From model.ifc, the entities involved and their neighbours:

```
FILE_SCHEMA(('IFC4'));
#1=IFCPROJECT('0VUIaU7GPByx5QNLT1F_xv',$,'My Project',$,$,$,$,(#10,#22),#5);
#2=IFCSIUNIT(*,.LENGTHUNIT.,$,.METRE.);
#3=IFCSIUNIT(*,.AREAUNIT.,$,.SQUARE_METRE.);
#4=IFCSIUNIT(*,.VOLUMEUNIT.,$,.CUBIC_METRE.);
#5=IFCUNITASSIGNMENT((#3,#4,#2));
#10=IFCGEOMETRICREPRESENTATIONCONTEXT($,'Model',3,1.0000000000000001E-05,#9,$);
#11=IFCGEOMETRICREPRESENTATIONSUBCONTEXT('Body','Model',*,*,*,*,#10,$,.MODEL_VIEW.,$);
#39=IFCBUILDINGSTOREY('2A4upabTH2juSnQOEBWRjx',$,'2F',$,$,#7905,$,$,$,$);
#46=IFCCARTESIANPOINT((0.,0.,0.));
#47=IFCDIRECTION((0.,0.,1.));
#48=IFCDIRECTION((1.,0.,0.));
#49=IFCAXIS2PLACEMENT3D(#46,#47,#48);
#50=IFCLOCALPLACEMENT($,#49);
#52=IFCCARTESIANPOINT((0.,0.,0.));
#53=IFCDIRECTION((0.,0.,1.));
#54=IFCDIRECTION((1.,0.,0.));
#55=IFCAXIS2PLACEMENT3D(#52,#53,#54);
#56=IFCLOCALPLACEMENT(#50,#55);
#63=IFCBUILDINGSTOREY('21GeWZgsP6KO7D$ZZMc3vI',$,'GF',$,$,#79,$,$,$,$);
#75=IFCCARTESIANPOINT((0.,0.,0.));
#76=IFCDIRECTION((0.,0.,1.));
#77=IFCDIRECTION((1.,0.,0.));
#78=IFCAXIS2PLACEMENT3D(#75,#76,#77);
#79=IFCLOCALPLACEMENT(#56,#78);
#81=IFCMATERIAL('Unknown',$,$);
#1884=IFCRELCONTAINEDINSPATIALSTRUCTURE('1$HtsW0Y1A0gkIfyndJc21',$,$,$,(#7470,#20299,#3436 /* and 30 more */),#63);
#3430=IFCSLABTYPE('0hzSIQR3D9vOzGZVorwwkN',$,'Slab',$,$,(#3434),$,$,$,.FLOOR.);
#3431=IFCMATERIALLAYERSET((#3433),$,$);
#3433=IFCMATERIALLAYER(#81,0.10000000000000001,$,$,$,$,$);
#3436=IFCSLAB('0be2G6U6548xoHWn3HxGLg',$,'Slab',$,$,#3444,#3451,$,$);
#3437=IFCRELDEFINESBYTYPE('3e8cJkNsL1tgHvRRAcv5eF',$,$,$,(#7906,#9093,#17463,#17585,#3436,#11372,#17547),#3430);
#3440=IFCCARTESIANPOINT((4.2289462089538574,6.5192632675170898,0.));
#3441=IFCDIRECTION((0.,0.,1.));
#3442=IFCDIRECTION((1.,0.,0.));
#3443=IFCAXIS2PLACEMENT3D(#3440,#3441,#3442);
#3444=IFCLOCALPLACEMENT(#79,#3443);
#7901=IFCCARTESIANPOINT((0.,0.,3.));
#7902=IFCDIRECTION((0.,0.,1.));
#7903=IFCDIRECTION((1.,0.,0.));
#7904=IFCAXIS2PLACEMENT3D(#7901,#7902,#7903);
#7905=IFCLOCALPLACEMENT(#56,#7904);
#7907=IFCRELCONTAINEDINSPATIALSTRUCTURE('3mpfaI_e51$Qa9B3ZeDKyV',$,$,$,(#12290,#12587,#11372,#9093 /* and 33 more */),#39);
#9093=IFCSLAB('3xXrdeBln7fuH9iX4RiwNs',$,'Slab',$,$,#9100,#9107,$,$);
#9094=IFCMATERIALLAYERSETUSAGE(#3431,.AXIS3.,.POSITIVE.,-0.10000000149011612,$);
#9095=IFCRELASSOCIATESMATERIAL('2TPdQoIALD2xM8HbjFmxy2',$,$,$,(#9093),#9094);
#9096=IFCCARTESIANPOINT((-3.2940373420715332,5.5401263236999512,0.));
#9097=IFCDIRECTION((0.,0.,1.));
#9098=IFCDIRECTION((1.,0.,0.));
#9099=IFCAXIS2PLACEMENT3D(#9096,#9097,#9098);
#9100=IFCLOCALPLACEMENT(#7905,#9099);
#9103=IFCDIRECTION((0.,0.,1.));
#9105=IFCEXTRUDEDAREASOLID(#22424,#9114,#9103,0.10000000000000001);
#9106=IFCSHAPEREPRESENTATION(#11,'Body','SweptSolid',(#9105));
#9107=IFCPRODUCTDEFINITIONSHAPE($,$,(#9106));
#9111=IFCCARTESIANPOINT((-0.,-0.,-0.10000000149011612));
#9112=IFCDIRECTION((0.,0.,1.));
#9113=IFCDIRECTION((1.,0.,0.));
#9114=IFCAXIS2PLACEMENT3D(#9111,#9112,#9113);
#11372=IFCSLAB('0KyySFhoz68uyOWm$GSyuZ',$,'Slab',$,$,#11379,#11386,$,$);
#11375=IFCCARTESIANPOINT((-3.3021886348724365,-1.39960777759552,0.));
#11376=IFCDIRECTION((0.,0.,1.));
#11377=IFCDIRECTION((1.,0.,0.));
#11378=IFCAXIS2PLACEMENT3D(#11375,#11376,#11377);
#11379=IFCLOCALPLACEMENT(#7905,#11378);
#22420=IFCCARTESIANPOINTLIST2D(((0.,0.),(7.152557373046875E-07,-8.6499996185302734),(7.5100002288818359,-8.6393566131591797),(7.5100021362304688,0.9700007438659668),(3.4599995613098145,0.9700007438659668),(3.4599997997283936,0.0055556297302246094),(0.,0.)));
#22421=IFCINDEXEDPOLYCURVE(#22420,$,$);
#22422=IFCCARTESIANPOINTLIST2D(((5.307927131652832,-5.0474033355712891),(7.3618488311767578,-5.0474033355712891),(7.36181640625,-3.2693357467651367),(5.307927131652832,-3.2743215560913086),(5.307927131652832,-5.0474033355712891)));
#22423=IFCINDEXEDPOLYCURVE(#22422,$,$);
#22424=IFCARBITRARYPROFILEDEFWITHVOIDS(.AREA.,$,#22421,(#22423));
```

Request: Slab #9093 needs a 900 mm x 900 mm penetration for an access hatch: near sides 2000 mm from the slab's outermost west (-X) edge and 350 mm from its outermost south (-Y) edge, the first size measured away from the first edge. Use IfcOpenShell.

```python
import numpy as np
import ifcopenshell
import ifcopenshell.api.feature
import ifcopenshell.api.geometry
import ifcopenshell.api.root
import ifcopenshell.geom
import ifcopenshell.util.placement
import ifcopenshell.util.representation
import ifcopenshell.util.shape
import ifcopenshell.util.unit

model = ifcopenshell.open("model.ifc")
unit_scale = ifcopenshell.util.unit.calculate_unit_scale(model)
settings = ifcopenshell.geom.settings()


def volume(element):
    """Net volume in cubic metres, openings subtracted."""
    shape = ifcopenshell.geom.create_shape(settings, element)
    return ifcopenshell.util.shape.get_volume(shape.geometry)


slab = model.by_id(9093)
before = volume(slab)

# Extent in the slab's own axes, in metres. The edges named are its -X and -Y sides.
slab_shape = ifcopenshell.geom.create_shape(settings, slab)
vertices = ifcopenshell.util.shape.get_vertices(slab_shape.geometry)
x_min, y_min, bottom = vertices.min(axis=0)
top = vertices[:, 2].max()

opening = ifcopenshell.api.root.create_entity(model, ifc_class="IfcOpeningElement", name="Access hatch opening", predefined_type="OPENING")
context = ifcopenshell.util.representation.get_context(model, "Model", "Body", "MODEL_VIEW")
width, depth = 0.9, 0.9
outline = [(0.0, 0.0), (width, 0.0), (width, depth), (0.0, depth), (0.0, 0.0)]
# Overshoot both faces by 50 mm so the cut is clean.
shape = ifcopenshell.api.geometry.add_slab_representation(
    model, context=context, depth=top - bottom + 0.1, polyline=outline
)
ifcopenshell.api.geometry.assign_representation(model, product=opening, representation=shape)

matrix = ifcopenshell.util.placement.get_local_placement(slab.ObjectPlacement)
matrix[:, 3] = matrix @ np.append(np.array([x_min + 2, y_min + 0.35, bottom - 0.05]) / unit_scale, 1.0)
ifcopenshell.api.geometry.edit_object_placement(model, product=opening, matrix=matrix, is_si=False)
ifcopenshell.api.feature.add_feature(model, feature=opening, element=slab)

after = volume(slab)

print(f"slab volume {before:.3f} -> {after:.3f} m3")

model.write("model_v2.ifc")
```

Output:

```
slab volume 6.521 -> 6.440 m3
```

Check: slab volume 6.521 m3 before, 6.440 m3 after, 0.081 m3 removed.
